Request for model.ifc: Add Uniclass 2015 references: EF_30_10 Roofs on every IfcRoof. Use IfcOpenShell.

First a look at what the model holds.

```python
import ifcopenshell

model = ifcopenshell.open("model.ifc")
print(model.schema)
print("classifications:", [c.Name for c in model.by_type("IfcClassification")])
for ifc_class in ("IfcDoor", "IfcRoof", "IfcStair", "IfcWall", "IfcWindow"):
    print(ifc_class, len(model.by_type(ifc_class)))
```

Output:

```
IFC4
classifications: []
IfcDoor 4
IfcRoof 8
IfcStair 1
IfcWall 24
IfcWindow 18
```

```python
import ifcopenshell
import ifcopenshell.api.classification

model = ifcopenshell.open("model.ifc")

system = ifcopenshell.api.classification.add_classification(model, classification="Uniclass 2015")

codes = {
    "IfcRoof": ("EF_30_10", "Roofs"),
}
for ifc_class, (code, name) in codes.items():
    products = model.by_type(ifc_class)
    ifcopenshell.api.classification.add_reference(
        model, products=products, classification=system, identification=code, name=name
    )
    print(code, len(products))

model.write("model_v2.ifc")
```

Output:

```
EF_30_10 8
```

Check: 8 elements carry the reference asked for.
